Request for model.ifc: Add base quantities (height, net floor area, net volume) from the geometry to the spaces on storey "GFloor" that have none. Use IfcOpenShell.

First a look at what the model holds.

```python
import ifcopenshell
import ifcopenshell.util.element
import ifcopenshell.util.unit

model = ifcopenshell.open("model.ifc")
print(model.schema)
for unit_type in ("LENGTHUNIT", "AREAUNIT", "VOLUMEUNIT"):
    print(unit_type, ifcopenshell.util.unit.calculate_unit_scale(model, unit_type))
storey = next(s for s in model.by_type("IfcBuildingStorey") if s.Name == "GFloor")
spaces = [e for e in ifcopenshell.util.element.get_decomposition(storey) if e.is_a("IfcSpace")]
for e in sorted(spaces, key=lambda e: e.id()):
    print(e.id(), e.is_a(), e.Name, list(ifcopenshell.util.element.get_psets(e, qtos_only=True)), sep=" | ")
```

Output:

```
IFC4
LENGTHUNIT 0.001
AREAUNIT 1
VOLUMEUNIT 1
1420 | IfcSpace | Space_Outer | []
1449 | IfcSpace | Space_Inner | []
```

```python
import ifcopenshell
import ifcopenshell.api.pset
import ifcopenshell.geom
import ifcopenshell.util.element
import ifcopenshell.util.shape
import ifcopenshell.util.unit

model = ifcopenshell.open("model.ifc")
unit_scale = ifcopenshell.util.unit.calculate_unit_scale(model)
area_scale = ifcopenshell.util.unit.calculate_unit_scale(model, "AREAUNIT")
volume_scale = ifcopenshell.util.unit.calculate_unit_scale(model, "VOLUMEUNIT")
settings = ifcopenshell.geom.settings()

storey = next(s for s in model.by_type("IfcBuildingStorey") if s.Name == "GFloor")
spaces = [e for e in ifcopenshell.util.element.get_decomposition(storey) if e.is_a("IfcSpace")]

for e in sorted(spaces, key=lambda e: e.id()):
    if ifcopenshell.util.element.get_psets(e, qtos_only=True, should_inherit=False):
        continue
    # Geometry comes back in metres, in the element's own axes.
    shape = ifcopenshell.geom.create_shape(settings, e)
    values = {
        "Height": ifcopenshell.util.shape.get_z(shape.geometry) / unit_scale,
        "NetFloorArea": ifcopenshell.util.shape.get_footprint_area(shape.geometry) / area_scale,
        "NetVolume": ifcopenshell.util.shape.get_volume(shape.geometry) / volume_scale,
    }
    qto = ifcopenshell.api.pset.add_qto(model, product=e, name="Qto_SpaceBaseQuantities")
    ifcopenshell.api.pset.edit_qto(model, qto=qto, properties=values)
    print(e.id(), {k: round(v, 3) for k, v in values.items()})

model.write("model_edited.ifc")
```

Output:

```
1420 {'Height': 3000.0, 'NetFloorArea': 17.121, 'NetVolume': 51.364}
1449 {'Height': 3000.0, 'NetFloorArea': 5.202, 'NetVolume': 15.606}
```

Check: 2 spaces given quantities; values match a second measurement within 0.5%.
